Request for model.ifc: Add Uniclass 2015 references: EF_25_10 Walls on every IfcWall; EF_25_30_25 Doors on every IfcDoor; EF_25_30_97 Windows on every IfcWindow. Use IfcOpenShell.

First a look at what the model holds.

```python
import ifcopenshell

model = ifcopenshell.open("model.ifc")
print(model.schema)
print("classifications:", [c.Name for c in model.by_type("IfcClassification")])
for ifc_class in ("IfcDoor", "IfcRoof", "IfcStair", "IfcWall", "IfcWindow"):
    print(ifc_class, len(model.by_type(ifc_class)))
```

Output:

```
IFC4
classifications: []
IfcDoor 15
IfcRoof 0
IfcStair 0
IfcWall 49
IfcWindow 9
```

```python
import ifcopenshell
import ifcopenshell.api.classification

model = ifcopenshell.open("model.ifc")

system = ifcopenshell.api.classification.add_classification(model, classification="Uniclass 2015")

codes = {
    "IfcWall": ("EF_25_10", "Walls"),
    "IfcDoor": ("EF_25_30_25", "Doors"),
    "IfcWindow": ("EF_25_30_97", "Windows"),
}
for ifc_class, (code, name) in codes.items():
    products = model.by_type(ifc_class)
    ifcopenshell.api.classification.add_reference(
        model, products=products, classification=system, identification=code, name=name
    )
    print(code, len(products))

model.write("model_updated.ifc")
```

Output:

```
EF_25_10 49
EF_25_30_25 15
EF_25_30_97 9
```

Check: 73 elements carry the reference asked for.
